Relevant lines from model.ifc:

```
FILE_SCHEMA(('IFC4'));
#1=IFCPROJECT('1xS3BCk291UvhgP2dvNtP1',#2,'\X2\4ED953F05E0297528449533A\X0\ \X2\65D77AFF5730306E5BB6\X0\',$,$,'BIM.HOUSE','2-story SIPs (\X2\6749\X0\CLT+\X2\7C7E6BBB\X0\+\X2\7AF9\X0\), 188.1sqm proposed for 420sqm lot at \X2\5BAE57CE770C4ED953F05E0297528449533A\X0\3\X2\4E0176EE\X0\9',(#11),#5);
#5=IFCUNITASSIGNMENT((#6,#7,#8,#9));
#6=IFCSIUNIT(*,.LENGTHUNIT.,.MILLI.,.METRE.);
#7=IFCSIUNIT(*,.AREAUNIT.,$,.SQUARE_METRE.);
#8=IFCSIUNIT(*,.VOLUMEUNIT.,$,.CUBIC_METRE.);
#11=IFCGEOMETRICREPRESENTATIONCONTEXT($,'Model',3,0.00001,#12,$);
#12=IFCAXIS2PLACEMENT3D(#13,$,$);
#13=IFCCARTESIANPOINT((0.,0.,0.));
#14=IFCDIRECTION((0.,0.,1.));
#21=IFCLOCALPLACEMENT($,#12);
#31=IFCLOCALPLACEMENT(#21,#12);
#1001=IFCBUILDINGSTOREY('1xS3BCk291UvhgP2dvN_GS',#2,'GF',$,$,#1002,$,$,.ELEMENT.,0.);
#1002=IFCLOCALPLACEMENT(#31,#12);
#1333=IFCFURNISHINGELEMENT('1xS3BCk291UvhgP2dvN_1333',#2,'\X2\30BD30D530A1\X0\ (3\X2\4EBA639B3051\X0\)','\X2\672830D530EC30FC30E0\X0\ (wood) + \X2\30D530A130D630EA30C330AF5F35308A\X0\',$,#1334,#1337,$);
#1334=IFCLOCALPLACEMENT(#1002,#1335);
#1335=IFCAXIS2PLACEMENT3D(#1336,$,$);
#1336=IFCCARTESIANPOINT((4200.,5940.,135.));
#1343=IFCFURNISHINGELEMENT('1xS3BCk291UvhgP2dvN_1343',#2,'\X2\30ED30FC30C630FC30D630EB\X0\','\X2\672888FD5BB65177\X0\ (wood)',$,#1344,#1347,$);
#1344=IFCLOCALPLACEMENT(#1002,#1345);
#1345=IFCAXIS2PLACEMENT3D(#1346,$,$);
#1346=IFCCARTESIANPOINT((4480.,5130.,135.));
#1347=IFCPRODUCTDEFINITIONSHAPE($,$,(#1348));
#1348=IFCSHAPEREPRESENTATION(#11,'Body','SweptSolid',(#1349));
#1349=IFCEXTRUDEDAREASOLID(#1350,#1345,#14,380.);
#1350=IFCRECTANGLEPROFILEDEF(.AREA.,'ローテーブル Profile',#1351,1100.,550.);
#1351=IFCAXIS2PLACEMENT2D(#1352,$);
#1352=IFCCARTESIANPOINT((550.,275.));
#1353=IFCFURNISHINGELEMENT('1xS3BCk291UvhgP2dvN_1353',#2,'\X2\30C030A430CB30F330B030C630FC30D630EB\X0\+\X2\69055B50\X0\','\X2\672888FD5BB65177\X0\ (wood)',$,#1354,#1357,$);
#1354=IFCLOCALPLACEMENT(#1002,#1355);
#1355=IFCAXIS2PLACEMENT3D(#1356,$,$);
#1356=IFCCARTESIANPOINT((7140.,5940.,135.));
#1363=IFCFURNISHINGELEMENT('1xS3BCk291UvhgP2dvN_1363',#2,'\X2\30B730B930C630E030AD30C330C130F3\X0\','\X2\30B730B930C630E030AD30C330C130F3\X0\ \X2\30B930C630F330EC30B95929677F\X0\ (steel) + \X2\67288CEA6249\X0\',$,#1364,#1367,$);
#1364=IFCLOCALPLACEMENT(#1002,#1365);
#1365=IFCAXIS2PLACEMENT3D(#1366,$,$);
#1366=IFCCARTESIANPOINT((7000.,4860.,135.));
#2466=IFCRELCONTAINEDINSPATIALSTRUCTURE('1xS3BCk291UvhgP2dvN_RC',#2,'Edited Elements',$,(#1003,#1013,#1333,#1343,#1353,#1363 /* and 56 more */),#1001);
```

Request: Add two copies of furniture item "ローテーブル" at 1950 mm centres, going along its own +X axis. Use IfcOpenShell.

```python
import ifcopenshell
import ifcopenshell.api.geometry
import ifcopenshell.api.root
import ifcopenshell.util.element
import ifcopenshell.util.placement

model = ifcopenshell.open("model.ifc")


def reuse_history(source, copy):
    """copy_class also copies each property set's owner history, people and application; keep the originals."""
    for rel in copy.IsDefinedBy:
        if rel.is_a("IfcRelDefinesByProperties") and (history := rel.RelatingPropertyDefinition.OwnerHistory):
            rel.RelatingPropertyDefinition.OwnerHistory = source.OwnerHistory
            ifcopenshell.util.element.remove_deep2(model, history)


source = model.by_guid("1xS3BCk291UvhgP2dvN_1343")
base = ifcopenshell.util.placement.get_local_placement(source.ObjectPlacement)
step = base[:3, 0] * 1950.0

for i in range(1, 3):
    copy = ifcopenshell.api.root.copy_class(model, product=source)
    copy.Representation = ifcopenshell.util.element.copy_deep(
        model, source.Representation, exclude=["IfcGeometricRepresentationContext", "IfcRepresentationMap"]
    )
    reuse_history(source, copy)
    matrix = base.copy()
    matrix[:3, 3] += i * step
    print("added at", matrix[:3, 3].round(3) + 0.0)
    ifcopenshell.api.geometry.edit_object_placement(model, product=copy, matrix=matrix, is_si=False)

model.write("model-out.ifc")
```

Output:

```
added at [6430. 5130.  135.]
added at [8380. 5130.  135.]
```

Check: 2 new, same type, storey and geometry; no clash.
